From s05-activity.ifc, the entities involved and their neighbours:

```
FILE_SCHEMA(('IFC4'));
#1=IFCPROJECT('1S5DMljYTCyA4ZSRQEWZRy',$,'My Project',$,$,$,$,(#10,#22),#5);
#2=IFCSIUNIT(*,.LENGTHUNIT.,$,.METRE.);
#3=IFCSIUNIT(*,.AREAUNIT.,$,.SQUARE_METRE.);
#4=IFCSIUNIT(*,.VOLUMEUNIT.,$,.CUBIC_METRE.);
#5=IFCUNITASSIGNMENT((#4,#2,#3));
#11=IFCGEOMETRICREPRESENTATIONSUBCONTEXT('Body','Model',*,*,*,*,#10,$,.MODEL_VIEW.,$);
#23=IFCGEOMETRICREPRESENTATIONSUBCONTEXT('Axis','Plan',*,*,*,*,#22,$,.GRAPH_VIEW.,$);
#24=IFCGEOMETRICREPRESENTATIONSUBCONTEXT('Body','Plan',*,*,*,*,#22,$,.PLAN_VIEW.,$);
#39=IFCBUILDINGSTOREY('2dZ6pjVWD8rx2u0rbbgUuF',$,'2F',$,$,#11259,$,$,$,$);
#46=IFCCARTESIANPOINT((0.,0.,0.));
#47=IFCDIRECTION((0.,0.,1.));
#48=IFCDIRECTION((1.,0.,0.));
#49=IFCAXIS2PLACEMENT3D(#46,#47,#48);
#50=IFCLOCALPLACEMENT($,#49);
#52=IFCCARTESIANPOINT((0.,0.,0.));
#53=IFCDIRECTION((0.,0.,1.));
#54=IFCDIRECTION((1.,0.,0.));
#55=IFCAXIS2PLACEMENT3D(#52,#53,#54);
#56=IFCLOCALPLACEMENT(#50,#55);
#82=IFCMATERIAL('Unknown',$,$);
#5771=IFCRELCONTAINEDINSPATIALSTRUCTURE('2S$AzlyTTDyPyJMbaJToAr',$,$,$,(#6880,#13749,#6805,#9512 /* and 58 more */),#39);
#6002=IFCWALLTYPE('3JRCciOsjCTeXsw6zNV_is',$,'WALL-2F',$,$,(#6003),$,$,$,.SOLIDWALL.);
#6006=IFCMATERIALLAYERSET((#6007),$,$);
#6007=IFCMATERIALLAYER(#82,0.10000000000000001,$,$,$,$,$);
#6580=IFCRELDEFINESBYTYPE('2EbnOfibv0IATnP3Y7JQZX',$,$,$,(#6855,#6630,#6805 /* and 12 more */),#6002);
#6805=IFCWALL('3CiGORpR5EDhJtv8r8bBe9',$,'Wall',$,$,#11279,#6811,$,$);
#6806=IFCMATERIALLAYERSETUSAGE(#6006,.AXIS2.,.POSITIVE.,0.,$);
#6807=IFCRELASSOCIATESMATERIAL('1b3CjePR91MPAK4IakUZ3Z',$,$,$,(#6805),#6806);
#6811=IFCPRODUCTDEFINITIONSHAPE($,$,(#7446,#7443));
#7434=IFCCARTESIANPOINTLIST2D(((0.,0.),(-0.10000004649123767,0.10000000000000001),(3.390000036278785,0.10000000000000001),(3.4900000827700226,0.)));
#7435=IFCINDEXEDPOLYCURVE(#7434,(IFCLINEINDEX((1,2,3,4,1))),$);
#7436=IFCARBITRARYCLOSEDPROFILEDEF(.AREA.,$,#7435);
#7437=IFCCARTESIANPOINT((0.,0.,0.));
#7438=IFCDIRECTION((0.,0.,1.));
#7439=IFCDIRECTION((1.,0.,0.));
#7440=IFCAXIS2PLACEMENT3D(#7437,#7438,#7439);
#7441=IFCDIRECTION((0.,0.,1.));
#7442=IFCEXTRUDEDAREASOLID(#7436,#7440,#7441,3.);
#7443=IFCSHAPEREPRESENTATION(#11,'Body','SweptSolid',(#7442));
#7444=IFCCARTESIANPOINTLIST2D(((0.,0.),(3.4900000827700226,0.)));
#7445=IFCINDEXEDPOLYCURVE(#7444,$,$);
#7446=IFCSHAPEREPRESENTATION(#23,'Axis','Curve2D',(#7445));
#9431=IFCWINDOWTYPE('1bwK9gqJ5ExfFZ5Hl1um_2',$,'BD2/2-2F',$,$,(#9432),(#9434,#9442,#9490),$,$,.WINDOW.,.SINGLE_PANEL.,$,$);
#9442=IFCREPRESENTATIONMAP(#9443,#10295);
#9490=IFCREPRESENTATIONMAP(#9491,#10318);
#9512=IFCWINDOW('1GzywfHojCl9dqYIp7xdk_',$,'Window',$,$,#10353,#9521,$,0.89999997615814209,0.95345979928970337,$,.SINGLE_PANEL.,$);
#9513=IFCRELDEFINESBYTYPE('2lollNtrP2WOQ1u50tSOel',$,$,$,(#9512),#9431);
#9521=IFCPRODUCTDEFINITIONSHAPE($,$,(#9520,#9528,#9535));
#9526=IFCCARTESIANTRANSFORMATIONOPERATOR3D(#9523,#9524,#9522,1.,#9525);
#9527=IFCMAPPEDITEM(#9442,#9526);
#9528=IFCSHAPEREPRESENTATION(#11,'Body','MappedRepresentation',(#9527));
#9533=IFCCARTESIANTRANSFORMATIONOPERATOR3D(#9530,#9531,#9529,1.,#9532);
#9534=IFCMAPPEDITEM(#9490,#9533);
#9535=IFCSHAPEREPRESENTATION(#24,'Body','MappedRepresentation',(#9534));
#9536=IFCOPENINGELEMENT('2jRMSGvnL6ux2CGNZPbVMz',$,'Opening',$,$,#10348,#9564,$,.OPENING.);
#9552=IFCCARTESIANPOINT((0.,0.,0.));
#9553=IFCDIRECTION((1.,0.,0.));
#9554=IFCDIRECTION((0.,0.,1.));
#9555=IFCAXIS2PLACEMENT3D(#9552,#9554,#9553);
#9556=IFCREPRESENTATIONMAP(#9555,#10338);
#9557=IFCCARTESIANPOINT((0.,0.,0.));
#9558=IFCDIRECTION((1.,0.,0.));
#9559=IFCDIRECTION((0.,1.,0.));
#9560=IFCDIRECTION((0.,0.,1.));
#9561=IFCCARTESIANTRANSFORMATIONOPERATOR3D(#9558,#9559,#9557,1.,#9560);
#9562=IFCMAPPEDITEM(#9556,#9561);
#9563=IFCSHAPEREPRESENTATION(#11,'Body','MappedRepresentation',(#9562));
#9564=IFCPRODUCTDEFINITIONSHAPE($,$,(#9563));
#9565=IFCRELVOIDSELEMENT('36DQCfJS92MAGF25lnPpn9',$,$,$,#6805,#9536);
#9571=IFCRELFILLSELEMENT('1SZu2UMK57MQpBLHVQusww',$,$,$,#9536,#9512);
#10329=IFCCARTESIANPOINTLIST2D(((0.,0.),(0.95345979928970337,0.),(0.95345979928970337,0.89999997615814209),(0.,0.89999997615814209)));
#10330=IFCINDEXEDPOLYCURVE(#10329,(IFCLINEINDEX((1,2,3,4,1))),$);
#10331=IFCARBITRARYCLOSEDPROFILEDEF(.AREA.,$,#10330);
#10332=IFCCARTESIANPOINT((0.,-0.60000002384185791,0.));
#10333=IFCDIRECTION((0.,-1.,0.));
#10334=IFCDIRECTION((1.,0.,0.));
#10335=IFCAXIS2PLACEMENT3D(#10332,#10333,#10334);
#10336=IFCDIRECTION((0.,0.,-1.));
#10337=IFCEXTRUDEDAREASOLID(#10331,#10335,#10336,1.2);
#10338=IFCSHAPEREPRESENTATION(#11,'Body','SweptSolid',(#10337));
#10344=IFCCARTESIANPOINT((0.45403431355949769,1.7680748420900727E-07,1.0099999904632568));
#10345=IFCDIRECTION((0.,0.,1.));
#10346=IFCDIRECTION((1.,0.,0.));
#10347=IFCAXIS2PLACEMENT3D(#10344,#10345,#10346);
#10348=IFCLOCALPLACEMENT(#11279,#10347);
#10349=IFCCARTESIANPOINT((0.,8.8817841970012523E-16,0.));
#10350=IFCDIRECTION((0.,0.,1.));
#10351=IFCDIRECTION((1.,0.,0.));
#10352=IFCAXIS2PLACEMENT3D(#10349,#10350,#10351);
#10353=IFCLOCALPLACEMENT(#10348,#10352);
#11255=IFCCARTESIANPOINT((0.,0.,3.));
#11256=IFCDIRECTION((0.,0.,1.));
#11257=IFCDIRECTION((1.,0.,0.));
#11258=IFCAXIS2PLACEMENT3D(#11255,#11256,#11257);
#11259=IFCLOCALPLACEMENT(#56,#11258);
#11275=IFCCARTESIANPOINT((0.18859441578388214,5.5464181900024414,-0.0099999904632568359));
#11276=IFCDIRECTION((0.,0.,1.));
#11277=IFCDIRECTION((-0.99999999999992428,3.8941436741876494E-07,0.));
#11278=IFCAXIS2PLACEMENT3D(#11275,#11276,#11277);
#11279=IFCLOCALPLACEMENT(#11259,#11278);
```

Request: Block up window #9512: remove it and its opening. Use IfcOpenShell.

```python
import ifcopenshell
import ifcopenshell.api.feature
import ifcopenshell.api.root
import ifcopenshell.geom
import ifcopenshell.util.shape

model = ifcopenshell.open("s05-activity.ifc")
settings = ifcopenshell.geom.settings()


def volume(element):
    """Net volume in cubic metres, openings subtracted."""
    shape = ifcopenshell.geom.create_shape(settings, element)
    return ifcopenshell.util.shape.get_volume(shape.geometry)


window = model.by_guid("1GzywfHojCl9dqYIp7xdk_")
opening = window.FillsVoids[0].RelatingOpeningElement
wall = opening.VoidsElements[0].RelatingBuildingElement
before = volume(wall)

ifcopenshell.api.root.remove_product(model, product=window)
ifcopenshell.api.feature.remove_feature(model, feature=opening)

after = volume(wall)

print(f"wall volume {before:.3f} -> {after:.3f} m3")

model.write("s05-activity_updated.ifc")
```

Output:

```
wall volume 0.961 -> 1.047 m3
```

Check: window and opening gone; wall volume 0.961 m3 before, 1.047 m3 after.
